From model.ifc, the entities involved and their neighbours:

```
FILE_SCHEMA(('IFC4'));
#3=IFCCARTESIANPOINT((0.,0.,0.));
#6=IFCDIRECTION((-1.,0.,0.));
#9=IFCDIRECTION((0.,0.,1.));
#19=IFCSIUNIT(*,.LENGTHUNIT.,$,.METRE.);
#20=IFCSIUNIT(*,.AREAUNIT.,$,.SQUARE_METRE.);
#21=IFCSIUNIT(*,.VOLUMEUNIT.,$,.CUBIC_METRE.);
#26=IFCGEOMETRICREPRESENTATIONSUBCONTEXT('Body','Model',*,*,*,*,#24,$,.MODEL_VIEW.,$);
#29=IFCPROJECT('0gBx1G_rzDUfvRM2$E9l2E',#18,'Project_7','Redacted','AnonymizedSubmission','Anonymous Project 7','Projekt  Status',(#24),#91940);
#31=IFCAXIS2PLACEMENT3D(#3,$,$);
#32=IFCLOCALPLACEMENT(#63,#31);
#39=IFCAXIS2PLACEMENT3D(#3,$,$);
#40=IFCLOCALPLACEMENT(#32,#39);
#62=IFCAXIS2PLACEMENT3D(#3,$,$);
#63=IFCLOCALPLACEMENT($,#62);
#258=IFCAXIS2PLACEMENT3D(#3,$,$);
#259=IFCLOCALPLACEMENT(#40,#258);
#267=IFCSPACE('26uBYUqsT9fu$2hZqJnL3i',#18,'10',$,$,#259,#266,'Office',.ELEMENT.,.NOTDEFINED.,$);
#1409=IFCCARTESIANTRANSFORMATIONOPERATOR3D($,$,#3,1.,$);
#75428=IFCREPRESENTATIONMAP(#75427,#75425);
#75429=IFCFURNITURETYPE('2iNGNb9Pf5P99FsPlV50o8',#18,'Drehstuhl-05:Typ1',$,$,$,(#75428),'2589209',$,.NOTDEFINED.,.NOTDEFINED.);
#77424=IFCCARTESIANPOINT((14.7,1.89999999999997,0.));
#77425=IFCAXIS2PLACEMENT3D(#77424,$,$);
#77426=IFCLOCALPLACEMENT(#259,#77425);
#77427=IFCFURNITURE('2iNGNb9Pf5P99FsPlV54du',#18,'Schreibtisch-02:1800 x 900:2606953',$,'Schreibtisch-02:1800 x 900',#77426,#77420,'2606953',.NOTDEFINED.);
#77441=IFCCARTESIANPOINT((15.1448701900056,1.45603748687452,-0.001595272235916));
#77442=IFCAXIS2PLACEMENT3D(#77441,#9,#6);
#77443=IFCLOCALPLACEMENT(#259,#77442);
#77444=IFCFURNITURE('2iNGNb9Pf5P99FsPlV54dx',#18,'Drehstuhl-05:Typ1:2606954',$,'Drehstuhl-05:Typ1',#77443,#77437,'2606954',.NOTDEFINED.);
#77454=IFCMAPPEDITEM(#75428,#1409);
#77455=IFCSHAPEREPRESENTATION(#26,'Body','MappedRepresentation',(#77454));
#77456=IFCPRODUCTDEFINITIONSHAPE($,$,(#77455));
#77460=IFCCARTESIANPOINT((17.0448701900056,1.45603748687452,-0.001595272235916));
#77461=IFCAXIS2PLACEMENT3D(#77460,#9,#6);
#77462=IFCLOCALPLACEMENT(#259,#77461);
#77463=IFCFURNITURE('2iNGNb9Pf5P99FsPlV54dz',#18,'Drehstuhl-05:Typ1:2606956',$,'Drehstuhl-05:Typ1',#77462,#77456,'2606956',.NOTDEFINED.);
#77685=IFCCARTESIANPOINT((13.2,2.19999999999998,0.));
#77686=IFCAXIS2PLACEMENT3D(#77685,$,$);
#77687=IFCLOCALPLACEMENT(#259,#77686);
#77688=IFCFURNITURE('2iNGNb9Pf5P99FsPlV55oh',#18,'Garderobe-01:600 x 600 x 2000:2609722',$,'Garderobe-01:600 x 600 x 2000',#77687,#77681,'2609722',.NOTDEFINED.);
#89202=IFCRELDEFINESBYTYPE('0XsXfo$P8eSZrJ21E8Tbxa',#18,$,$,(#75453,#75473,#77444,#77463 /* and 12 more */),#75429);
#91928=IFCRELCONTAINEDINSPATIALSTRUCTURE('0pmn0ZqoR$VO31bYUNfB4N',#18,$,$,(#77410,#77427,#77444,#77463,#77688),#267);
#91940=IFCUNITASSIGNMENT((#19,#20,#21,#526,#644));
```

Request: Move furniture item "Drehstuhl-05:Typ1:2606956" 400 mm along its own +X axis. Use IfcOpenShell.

```python
import ifcopenshell
import ifcopenshell.api.geometry
import ifcopenshell.util.placement

model = ifcopenshell.open("model.ifc")

item = model.by_id(77463)
matrix = ifcopenshell.util.placement.get_local_placement(item.ObjectPlacement)
matrix[:3, 3] += matrix[:3, 0] * 0.4
ifcopenshell.api.geometry.edit_object_placement(model, product=item, matrix=matrix, is_si=False)

print(ifcopenshell.util.placement.get_local_placement(item.ObjectPlacement).round(3) + 0.0)

model.write("model_updated.ifc")
```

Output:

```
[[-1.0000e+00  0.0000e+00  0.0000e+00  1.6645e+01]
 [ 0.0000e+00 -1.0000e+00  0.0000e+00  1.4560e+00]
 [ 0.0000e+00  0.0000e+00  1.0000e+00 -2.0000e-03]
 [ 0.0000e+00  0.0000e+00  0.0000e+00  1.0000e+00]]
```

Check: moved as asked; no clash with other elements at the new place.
